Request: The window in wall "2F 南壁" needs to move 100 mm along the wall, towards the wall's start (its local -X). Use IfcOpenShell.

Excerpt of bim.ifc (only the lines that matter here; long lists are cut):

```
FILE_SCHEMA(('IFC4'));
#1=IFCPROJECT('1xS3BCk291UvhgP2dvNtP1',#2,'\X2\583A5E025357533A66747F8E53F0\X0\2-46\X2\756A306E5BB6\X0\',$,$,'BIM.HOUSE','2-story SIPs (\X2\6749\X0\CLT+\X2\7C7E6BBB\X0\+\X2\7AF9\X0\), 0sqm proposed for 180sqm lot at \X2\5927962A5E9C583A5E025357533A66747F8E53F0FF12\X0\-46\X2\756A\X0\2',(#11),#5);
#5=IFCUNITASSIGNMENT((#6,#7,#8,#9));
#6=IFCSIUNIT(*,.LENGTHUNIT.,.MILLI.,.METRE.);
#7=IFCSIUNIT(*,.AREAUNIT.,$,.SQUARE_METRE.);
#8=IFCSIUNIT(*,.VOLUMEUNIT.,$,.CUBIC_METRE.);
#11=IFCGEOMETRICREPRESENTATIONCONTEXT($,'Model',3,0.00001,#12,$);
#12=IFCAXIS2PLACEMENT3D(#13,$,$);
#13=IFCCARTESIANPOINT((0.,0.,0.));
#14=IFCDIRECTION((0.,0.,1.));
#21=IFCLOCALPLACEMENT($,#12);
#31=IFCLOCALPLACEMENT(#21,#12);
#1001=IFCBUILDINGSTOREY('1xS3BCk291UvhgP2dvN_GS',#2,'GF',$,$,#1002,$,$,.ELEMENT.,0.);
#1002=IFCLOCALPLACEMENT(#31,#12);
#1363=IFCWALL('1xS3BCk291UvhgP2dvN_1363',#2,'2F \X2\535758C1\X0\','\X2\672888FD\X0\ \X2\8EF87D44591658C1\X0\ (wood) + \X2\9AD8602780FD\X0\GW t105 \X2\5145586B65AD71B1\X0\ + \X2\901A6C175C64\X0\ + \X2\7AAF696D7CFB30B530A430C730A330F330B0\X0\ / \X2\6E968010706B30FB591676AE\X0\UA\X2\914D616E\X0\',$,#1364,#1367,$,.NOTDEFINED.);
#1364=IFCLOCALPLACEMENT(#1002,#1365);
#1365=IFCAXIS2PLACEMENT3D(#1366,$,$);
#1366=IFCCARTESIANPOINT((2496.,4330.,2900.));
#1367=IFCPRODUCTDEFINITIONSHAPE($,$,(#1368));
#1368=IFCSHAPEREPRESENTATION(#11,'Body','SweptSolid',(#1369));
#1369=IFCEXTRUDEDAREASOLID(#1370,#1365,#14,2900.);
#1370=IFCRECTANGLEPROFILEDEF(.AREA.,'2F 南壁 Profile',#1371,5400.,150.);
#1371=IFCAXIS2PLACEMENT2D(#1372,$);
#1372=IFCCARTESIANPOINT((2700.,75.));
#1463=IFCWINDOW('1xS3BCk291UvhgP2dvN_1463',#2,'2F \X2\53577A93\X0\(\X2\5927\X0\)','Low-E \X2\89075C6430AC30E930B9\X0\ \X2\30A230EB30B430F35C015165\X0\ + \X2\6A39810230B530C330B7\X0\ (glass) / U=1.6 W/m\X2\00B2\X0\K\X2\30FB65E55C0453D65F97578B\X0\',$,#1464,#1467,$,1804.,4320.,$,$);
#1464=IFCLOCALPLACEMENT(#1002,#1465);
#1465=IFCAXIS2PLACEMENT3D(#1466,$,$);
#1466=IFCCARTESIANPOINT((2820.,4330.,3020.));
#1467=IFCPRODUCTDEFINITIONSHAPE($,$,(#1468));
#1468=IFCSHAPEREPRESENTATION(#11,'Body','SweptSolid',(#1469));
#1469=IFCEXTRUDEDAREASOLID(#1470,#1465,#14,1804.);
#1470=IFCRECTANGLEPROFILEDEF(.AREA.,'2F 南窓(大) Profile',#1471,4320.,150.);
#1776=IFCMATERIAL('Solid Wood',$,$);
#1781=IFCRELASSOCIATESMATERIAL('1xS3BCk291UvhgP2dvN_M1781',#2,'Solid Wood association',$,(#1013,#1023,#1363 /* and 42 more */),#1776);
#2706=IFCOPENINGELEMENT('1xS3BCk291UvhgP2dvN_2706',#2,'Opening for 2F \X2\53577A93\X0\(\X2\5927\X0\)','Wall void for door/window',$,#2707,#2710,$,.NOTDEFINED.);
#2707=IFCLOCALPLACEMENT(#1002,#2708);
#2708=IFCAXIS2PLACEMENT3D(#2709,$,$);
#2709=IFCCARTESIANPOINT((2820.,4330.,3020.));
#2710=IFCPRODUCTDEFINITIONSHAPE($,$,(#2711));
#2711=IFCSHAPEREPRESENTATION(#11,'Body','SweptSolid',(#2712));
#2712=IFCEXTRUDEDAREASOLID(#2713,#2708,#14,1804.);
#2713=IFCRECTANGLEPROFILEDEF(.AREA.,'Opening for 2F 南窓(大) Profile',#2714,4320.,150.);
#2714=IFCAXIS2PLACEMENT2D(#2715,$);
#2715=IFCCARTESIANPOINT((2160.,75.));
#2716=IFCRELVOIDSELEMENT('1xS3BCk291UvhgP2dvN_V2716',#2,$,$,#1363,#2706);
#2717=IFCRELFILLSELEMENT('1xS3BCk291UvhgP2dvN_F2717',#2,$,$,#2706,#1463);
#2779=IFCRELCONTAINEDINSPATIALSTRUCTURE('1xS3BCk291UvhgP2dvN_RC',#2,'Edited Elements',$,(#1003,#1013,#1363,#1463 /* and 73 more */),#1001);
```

```python
import ifcopenshell
import ifcopenshell.api.geometry
import ifcopenshell.util.placement
import ifcopenshell.util.unit

model = ifcopenshell.open("bim.ifc")
unit_scale = ifcopenshell.util.unit.calculate_unit_scale(model)

window = model.by_guid("1xS3BCk291UvhgP2dvN_1463")
opening = window.FillsVoids[0].RelatingOpeningElement
wall = opening.VoidsElements[0].RelatingBuildingElement

wall_matrix = ifcopenshell.util.placement.get_local_placement(wall.ObjectPlacement)
shift = wall_matrix[:3, 0] * -0.1 / unit_scale
before = ifcopenshell.util.placement.get_local_placement(window.ObjectPlacement)[:3, 3].copy()

# The window is not placed relative to its opening, so move both.
for product in (opening, window):
    matrix = ifcopenshell.util.placement.get_local_placement(product.ObjectPlacement)
    matrix[:3, 3] += shift
    ifcopenshell.api.geometry.edit_object_placement(model, product=product, matrix=matrix, is_si=False)

after = ifcopenshell.util.placement.get_local_placement(window.ObjectPlacement)[:3, 3]
print("window moved by", (after - before).round(3) + 0.0)

model.write("bim_updated.ifc")
```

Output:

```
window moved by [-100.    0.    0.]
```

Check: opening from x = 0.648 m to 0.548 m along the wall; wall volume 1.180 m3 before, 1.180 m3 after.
